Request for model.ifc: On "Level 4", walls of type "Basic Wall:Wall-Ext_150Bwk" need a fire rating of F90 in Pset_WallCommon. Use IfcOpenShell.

First a look at what the model holds.

```python
import ifcopenshell
import ifcopenshell.util.element

model = ifcopenshell.open("model.ifc")
print(model.schema)
storey = next(s for s in model.by_type("IfcBuildingStorey") if s.Name == "Level 4")
walls = [e for e in ifcopenshell.util.element.get_decomposition(storey) if e.is_a("IfcWall")]
seen = {}
for e in walls:
    element_type = ifcopenshell.util.element.get_type(e)
    key = (element_type.Name if element_type != e and element_type else None, ifcopenshell.util.element.get_pset(e, "Pset_WallCommon", "FireRating"))
    seen[key] = seen.get(key, 0) + 1
for (name, value), count in sorted(seen.items(), key=str):
    print(count, "x", name, "|", value)
```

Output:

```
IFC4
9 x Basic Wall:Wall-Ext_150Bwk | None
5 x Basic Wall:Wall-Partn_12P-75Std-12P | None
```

```python
import ifcopenshell
import ifcopenshell.api.pset
import ifcopenshell.util.element

model = ifcopenshell.open("model.ifc")

storey = next(s for s in model.by_type("IfcBuildingStorey") if s.Name == "Level 4")
walls = [e for e in ifcopenshell.util.element.get_decomposition(storey) if e.is_a("IfcWall")]

count = 0
for e in walls:
    element_type = ifcopenshell.util.element.get_type(e)
    if element_type in (None, e) or element_type.Name != "Basic Wall:Wall-Ext_150Bwk":
        continue
    # add_pset returns the element's existing set when there is one.
    pset = ifcopenshell.api.pset.add_pset(model, product=e, name="Pset_WallCommon")
    ifcopenshell.api.pset.edit_pset(model, pset=pset, properties={"FireRating": "F90"})
    count += 1

print(count, "walls updated")

model.write("model_updated.ifc")
```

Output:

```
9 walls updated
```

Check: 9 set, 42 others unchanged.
